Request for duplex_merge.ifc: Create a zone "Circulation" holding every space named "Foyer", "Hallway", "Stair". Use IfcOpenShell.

First a look at what the model holds.

```python
import ifcopenshell

model = ifcopenshell.open("duplex_merge.ifc")
print(model.schema)
seen = {}
for space in model.by_type("IfcSpace"):
    seen[space.LongName] = seen.get(space.LongName, 0) + 1
for name, count in sorted(seen.items(), key=str):
    print(count, "x", name)
print("zones:", [z.Name for z in model.by_type("IfcZone")][:20])
```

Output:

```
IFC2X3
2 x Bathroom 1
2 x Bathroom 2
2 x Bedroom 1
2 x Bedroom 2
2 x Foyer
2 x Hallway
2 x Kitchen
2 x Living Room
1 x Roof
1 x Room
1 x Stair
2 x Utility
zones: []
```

```python
import ifcopenshell
import ifcopenshell.api.group
import ifcopenshell.api.root

model = ifcopenshell.open("duplex_merge.ifc")

names = {"Foyer", "Hallway", "Stair"}
spaces = [s for s in model.by_type("IfcSpace") if s.LongName in names]

zone = ifcopenshell.api.root.create_entity(model, ifc_class="IfcZone", name="Circulation")
ifcopenshell.api.group.assign_group(model, products=spaces, group=zone)
print(len(spaces), "spaces in", zone.Name)

model.write("duplex_merge_updated.ifc")
```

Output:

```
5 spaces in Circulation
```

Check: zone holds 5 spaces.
